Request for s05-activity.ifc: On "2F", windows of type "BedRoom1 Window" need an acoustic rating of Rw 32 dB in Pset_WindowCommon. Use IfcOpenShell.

First a look at what the model holds.

```python
import ifcopenshell
import ifcopenshell.util.element

model = ifcopenshell.open("s05-activity.ifc")
print(model.schema)
storey = next(s for s in model.by_type("IfcBuildingStorey") if s.Name == "2F")
windows = [e for e in ifcopenshell.util.element.get_decomposition(storey) if e.is_a("IfcWindow")]
seen = {}
for e in windows:
    element_type = ifcopenshell.util.element.get_type(e)
    key = (element_type.Name if element_type != e and element_type else None, ifcopenshell.util.element.get_pset(e, "Pset_WindowCommon", "AcousticRating"))
    seen[key] = seen.get(key, 0) + 1
for (name, value), count in sorted(seen.items(), key=str):
    print(count, "x", name, "|", value)
```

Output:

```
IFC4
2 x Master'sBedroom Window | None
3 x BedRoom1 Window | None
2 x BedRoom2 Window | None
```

```python
import ifcopenshell
import ifcopenshell.api.pset
import ifcopenshell.util.element

model = ifcopenshell.open("s05-activity.ifc")

storey = next(s for s in model.by_type("IfcBuildingStorey") if s.Name == "2F")
windows = [e for e in ifcopenshell.util.element.get_decomposition(storey) if e.is_a("IfcWindow")]

count = 0
for e in windows:
    element_type = ifcopenshell.util.element.get_type(e)
    if element_type in (None, e) or element_type.Name != "BedRoom1 Window":
        continue
    # add_pset returns the element's existing set when there is one.
    pset = ifcopenshell.api.pset.add_pset(model, product=e, name="Pset_WindowCommon")
    ifcopenshell.api.pset.edit_pset(model, pset=pset, properties={"AcousticRating": "Rw 32 dB"})
    count += 1

print(count, "windows updated")

model.write("s05-activity_v2.ifc")
```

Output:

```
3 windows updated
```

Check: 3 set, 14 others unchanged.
